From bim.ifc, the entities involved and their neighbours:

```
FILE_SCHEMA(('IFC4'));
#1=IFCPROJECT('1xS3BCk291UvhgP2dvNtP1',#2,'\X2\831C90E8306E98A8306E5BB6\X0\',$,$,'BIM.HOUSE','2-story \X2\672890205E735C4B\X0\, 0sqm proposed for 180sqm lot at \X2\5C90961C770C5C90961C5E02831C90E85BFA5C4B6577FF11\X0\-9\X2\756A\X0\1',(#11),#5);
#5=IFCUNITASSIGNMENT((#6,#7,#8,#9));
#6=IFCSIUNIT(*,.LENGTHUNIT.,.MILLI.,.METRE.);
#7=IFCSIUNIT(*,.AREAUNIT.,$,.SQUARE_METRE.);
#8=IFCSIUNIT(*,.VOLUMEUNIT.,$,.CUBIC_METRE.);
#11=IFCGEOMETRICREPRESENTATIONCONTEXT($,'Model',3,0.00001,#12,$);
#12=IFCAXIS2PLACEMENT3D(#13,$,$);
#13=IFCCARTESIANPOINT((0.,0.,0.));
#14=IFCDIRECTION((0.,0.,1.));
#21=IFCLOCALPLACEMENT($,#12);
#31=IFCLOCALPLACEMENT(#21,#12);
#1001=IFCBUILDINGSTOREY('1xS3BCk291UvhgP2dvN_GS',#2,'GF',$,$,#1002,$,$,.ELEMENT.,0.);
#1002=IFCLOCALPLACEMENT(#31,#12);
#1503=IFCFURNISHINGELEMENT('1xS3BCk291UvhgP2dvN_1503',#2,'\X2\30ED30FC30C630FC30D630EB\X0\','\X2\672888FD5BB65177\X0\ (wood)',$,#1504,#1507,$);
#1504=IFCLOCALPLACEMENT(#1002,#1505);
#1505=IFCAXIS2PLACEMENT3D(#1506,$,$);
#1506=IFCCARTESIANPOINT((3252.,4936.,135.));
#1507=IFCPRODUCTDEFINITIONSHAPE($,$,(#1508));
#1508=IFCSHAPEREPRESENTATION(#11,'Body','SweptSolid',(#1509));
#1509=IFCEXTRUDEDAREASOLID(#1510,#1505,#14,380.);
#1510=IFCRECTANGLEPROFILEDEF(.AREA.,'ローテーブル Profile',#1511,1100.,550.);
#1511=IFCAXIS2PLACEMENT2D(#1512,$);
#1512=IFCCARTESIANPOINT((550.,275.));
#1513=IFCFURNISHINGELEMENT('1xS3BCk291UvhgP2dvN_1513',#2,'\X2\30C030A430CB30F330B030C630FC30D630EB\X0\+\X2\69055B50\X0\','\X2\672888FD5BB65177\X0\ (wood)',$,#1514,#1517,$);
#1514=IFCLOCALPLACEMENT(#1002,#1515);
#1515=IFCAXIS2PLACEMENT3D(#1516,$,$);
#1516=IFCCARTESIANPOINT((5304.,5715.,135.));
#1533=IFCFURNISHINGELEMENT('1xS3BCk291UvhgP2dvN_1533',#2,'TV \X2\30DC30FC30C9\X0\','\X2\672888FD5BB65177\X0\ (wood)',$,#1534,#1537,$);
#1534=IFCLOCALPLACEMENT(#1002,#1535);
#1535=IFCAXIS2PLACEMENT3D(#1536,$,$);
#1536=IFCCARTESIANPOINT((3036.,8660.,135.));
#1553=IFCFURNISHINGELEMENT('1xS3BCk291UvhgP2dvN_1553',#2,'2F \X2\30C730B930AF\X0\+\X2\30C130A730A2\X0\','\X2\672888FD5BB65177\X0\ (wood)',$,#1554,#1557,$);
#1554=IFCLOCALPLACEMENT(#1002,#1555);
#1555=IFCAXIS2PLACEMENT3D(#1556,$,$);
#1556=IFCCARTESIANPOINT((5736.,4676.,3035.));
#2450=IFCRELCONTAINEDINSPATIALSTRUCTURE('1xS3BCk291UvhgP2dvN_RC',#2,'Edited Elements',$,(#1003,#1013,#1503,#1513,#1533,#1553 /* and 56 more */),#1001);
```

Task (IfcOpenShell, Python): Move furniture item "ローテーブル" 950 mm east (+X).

```python
import ifcopenshell
import ifcopenshell.api.geometry
import ifcopenshell.util.placement
import ifcopenshell.util.unit

model = ifcopenshell.open("bim.ifc")
unit_scale = ifcopenshell.util.unit.calculate_unit_scale(model)

item = model.by_guid("1xS3BCk291UvhgP2dvN_1503")
matrix = ifcopenshell.util.placement.get_local_placement(item.ObjectPlacement)
matrix[0, 3] += 0.95 / unit_scale
ifcopenshell.api.geometry.edit_object_placement(model, product=item, matrix=matrix, is_si=False)

print(ifcopenshell.util.placement.get_local_placement(item.ObjectPlacement).round(3) + 0.0)

model.write("bim_edited.ifc")
```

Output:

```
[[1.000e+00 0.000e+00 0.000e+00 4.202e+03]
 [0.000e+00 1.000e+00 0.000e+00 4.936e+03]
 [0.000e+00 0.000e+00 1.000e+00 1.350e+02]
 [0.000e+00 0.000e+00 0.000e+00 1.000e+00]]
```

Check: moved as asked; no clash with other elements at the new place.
